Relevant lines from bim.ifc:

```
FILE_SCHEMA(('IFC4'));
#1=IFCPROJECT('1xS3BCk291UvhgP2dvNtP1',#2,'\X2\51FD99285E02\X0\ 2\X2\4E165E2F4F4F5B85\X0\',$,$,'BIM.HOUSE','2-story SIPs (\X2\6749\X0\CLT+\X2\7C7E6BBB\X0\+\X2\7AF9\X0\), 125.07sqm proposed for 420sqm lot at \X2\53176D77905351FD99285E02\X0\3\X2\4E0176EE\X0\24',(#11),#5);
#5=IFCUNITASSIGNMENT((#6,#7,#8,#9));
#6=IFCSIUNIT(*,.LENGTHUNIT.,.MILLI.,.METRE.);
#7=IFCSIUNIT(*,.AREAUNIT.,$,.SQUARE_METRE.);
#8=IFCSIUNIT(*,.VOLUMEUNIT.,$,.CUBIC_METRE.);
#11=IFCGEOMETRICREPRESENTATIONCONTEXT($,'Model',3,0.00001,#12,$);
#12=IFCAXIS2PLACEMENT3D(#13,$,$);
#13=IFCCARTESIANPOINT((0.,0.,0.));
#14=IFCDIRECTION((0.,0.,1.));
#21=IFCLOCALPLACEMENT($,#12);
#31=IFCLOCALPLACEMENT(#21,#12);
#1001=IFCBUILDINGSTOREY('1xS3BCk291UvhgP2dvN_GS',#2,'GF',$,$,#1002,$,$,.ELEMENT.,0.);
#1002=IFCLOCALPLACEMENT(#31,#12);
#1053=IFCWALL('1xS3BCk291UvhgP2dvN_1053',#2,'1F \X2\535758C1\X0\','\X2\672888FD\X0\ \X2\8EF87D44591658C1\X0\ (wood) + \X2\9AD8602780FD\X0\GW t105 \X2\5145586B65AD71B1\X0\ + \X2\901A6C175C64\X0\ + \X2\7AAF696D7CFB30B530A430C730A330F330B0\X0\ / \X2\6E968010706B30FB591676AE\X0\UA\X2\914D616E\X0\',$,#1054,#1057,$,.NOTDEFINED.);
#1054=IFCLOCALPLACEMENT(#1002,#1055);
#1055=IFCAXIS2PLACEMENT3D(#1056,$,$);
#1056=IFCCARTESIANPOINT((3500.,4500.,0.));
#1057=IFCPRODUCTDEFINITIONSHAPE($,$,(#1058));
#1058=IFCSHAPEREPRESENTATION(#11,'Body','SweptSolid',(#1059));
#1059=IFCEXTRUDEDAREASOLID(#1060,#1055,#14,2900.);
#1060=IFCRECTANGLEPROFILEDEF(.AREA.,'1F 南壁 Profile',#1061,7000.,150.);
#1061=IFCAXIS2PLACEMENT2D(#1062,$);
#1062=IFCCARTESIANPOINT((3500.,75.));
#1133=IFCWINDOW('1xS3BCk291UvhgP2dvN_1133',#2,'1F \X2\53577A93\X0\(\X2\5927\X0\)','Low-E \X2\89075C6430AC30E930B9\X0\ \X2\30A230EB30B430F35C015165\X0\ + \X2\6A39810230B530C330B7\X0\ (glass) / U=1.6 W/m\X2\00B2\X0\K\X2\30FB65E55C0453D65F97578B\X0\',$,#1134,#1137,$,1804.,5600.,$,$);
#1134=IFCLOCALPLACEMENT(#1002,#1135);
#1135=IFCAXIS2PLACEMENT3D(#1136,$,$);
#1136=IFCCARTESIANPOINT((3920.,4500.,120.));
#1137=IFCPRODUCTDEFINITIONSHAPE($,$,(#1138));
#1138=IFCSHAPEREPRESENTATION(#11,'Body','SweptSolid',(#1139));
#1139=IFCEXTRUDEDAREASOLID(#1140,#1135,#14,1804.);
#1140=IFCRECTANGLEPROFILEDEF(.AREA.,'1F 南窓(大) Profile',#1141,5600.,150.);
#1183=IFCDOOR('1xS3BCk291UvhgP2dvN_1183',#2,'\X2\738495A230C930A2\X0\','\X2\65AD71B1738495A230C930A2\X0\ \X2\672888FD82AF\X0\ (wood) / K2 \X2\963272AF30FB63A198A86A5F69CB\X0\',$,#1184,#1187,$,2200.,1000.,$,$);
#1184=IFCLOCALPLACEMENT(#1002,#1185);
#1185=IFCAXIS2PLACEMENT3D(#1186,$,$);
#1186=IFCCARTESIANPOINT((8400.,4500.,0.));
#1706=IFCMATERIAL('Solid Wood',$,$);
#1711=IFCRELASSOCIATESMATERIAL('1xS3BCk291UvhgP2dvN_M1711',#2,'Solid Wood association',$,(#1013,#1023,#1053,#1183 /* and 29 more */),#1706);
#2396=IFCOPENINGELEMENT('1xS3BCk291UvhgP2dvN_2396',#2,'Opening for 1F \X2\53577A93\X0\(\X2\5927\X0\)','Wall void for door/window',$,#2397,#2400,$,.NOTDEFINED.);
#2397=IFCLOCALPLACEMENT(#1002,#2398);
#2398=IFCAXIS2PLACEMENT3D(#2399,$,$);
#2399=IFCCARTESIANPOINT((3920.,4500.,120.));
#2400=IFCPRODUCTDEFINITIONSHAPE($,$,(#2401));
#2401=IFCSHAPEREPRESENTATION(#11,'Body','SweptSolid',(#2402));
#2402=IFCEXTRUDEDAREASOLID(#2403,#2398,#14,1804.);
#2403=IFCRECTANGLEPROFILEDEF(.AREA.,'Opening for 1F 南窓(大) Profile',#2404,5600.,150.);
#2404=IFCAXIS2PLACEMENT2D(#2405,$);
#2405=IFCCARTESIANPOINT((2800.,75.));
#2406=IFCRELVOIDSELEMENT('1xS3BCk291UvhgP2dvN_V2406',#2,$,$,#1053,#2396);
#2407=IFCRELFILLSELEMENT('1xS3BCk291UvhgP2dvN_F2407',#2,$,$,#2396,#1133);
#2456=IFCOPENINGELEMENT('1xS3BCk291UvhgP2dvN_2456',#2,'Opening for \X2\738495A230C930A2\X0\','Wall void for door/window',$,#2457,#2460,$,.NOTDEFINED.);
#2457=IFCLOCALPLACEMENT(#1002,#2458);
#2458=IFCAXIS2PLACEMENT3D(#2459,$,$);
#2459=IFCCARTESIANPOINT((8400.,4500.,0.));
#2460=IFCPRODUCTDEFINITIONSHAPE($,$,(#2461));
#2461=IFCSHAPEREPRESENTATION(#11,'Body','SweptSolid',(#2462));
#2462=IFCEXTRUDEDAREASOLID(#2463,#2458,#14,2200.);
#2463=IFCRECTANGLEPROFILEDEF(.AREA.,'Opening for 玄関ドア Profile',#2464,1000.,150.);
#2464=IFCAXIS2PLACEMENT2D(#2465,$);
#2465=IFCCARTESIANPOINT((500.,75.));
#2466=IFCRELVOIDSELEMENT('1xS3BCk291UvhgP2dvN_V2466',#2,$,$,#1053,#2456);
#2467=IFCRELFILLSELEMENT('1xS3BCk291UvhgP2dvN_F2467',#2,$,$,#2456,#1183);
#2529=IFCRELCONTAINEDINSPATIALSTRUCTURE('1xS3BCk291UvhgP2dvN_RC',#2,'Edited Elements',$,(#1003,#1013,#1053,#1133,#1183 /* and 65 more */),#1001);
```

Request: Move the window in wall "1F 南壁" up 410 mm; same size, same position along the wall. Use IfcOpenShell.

```python
import numpy as np
import ifcopenshell
import ifcopenshell.api.geometry
import ifcopenshell.util.placement
import ifcopenshell.util.unit

model = ifcopenshell.open("bim.ifc")
unit_scale = ifcopenshell.util.unit.calculate_unit_scale(model)

window = model.by_guid("1xS3BCk291UvhgP2dvN_1133")
opening = window.FillsVoids[0].RelatingOpeningElement
dz = 410.0

shift = np.array([0.0, 0.0, dz])
# The window is not placed relative to its opening, so move both.
for product in (opening, window):
    matrix = ifcopenshell.util.placement.get_local_placement(product.ObjectPlacement)
    matrix[:3, 3] += shift
    ifcopenshell.api.geometry.edit_object_placement(model, product=product, matrix=matrix, is_si=False)

print(f"moved by {dz * unit_scale:+.3f} m")

model.write("bim_v2.ifc")
```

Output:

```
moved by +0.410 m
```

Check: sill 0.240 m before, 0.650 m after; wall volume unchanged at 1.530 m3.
